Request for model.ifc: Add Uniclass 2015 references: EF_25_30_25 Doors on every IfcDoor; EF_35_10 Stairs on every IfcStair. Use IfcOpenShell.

First a look at what the model holds.

```python
import ifcopenshell

model = ifcopenshell.open("model.ifc")
print(model.schema)
print("classifications:", [c.Name for c in model.by_type("IfcClassification")])
for ifc_class in ("IfcDoor", "IfcRoof", "IfcStair", "IfcWall", "IfcWindow"):
    print(ifc_class, len(model.by_type(ifc_class)))
```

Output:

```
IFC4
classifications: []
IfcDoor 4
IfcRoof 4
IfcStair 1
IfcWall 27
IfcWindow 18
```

```python
import ifcopenshell
import ifcopenshell.api.classification

model = ifcopenshell.open("model.ifc")

system = ifcopenshell.api.classification.add_classification(model, classification="Uniclass 2015")

codes = {
    "IfcDoor": ("EF_25_30_25", "Doors"),
    "IfcStair": ("EF_35_10", "Stairs"),
}
for ifc_class, (code, name) in codes.items():
    products = model.by_type(ifc_class)
    ifcopenshell.api.classification.add_reference(
        model, products=products, classification=system, identification=code, name=name
    )
    print(code, len(products))

model.write("model_updated.ifc")
```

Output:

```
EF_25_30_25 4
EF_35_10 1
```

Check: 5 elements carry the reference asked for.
